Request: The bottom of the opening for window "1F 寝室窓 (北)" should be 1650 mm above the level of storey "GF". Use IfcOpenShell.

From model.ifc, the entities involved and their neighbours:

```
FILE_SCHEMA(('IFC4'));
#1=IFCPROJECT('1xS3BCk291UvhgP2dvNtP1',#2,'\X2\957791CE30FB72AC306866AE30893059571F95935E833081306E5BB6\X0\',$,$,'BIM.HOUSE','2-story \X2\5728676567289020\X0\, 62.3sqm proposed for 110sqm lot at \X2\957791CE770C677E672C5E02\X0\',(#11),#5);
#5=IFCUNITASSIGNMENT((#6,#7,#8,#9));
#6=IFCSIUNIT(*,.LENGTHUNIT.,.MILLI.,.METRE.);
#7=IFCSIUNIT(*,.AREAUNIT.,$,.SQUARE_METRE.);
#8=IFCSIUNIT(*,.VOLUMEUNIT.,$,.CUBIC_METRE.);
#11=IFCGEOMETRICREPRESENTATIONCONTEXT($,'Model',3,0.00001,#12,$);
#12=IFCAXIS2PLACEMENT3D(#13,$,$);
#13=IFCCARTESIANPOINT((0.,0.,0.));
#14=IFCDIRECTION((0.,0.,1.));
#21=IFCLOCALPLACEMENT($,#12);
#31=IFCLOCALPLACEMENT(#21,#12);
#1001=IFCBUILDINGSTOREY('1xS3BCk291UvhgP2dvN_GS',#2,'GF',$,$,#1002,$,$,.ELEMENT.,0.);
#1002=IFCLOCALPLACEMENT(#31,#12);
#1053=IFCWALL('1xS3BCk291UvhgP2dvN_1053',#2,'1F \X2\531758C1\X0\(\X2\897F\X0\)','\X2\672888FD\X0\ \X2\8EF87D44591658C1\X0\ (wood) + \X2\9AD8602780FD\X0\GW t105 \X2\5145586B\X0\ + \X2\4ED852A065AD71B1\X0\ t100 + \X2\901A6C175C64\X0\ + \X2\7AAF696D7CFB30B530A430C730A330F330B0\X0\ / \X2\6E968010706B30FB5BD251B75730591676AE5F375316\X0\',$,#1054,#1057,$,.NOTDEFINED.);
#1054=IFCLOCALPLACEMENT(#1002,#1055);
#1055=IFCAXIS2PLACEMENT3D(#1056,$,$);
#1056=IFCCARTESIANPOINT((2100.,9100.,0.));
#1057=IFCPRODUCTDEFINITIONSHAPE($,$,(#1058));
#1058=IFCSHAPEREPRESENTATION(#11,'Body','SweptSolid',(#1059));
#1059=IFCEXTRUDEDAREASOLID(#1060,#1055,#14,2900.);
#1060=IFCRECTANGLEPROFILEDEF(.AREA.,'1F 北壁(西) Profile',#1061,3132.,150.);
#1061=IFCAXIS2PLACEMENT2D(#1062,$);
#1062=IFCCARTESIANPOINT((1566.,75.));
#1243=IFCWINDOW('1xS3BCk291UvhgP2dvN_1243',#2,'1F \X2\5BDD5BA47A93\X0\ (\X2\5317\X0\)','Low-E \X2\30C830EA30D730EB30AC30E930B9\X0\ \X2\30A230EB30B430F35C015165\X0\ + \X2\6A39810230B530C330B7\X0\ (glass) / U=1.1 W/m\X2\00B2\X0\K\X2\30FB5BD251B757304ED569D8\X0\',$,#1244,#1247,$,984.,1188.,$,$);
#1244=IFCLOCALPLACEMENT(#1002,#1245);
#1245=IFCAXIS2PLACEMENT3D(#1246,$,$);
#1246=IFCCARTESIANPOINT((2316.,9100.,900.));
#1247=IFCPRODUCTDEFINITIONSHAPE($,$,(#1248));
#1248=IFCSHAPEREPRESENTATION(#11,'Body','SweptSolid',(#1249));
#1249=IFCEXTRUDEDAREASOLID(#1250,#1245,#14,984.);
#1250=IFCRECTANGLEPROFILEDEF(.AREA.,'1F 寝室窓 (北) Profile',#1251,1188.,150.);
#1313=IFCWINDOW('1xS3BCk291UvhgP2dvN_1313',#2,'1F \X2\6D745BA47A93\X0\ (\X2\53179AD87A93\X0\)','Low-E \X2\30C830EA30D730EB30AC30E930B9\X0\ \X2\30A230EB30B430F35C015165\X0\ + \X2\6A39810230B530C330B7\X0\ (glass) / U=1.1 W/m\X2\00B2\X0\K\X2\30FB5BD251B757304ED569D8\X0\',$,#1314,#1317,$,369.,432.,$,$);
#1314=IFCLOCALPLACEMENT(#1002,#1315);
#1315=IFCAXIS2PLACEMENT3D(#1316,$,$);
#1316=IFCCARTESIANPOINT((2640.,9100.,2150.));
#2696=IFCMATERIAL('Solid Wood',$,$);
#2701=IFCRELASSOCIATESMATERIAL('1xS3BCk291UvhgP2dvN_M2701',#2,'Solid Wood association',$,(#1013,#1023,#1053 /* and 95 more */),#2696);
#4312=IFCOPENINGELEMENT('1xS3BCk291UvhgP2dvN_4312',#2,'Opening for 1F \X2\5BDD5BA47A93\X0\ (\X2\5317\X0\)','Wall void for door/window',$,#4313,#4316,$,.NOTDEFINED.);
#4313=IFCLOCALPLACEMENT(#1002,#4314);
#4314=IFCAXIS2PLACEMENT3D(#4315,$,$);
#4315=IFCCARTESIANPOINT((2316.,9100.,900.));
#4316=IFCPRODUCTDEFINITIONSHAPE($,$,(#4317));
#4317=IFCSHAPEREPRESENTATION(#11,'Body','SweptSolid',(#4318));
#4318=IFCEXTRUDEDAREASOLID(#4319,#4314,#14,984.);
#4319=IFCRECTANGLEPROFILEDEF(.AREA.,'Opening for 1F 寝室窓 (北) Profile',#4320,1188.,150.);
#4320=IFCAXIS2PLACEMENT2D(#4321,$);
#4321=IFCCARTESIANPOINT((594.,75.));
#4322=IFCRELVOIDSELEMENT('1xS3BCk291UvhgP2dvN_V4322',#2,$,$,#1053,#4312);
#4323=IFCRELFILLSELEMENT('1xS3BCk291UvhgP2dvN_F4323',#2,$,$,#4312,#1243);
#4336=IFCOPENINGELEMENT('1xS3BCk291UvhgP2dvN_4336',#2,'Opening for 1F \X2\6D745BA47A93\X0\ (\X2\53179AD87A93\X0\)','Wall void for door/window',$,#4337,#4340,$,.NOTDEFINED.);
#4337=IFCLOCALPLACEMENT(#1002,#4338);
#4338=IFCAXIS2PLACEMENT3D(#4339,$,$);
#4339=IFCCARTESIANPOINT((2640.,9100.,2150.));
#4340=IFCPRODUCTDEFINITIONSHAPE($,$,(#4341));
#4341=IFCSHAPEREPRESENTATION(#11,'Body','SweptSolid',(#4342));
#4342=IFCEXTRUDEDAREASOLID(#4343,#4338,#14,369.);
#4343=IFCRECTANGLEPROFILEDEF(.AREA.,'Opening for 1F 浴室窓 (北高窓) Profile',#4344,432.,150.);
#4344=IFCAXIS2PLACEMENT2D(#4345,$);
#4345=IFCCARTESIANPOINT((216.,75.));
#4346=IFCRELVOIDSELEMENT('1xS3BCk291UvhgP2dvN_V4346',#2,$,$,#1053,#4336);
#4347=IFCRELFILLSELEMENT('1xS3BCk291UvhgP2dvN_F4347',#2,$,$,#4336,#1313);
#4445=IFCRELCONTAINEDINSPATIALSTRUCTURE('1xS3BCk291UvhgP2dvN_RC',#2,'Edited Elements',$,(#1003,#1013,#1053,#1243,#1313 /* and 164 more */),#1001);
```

```python
import numpy as np
import ifcopenshell
import ifcopenshell.api.geometry
import ifcopenshell.geom
import ifcopenshell.util.element
import ifcopenshell.util.placement
import ifcopenshell.util.shape
import ifcopenshell.util.unit

model = ifcopenshell.open("model.ifc")
unit_scale = ifcopenshell.util.unit.calculate_unit_scale(model)

window = model.by_guid("1xS3BCk291UvhgP2dvN_1243")
opening = window.FillsVoids[0].RelatingOpeningElement
storey = ifcopenshell.util.element.get_container(window, ifc_class="IfcBuildingStorey")
level = ifcopenshell.util.placement.get_local_placement(storey.ObjectPlacement)[2, 3]

# The opening's origin need not be at the sill, so measure its lowest point.
shape = ifcopenshell.geom.create_shape(ifcopenshell.geom.settings(), opening)
bottom = ifcopenshell.util.shape.get_shape_bottom_elevation(shape, shape.geometry) / unit_scale
dz = level + 1650.0 - bottom

shift = np.array([0.0, 0.0, dz])
# The window is not placed relative to its opening, so move both.
for product in (opening, window):
    matrix = ifcopenshell.util.placement.get_local_placement(product.ObjectPlacement)
    matrix[:3, 3] += shift
    ifcopenshell.api.geometry.edit_object_placement(model, product=product, matrix=matrix, is_si=False)

print(f"moved by {dz * unit_scale:+.3f} m")

model.write("model_edited.ifc")
```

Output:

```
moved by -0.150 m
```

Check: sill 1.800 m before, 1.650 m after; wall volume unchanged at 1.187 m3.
